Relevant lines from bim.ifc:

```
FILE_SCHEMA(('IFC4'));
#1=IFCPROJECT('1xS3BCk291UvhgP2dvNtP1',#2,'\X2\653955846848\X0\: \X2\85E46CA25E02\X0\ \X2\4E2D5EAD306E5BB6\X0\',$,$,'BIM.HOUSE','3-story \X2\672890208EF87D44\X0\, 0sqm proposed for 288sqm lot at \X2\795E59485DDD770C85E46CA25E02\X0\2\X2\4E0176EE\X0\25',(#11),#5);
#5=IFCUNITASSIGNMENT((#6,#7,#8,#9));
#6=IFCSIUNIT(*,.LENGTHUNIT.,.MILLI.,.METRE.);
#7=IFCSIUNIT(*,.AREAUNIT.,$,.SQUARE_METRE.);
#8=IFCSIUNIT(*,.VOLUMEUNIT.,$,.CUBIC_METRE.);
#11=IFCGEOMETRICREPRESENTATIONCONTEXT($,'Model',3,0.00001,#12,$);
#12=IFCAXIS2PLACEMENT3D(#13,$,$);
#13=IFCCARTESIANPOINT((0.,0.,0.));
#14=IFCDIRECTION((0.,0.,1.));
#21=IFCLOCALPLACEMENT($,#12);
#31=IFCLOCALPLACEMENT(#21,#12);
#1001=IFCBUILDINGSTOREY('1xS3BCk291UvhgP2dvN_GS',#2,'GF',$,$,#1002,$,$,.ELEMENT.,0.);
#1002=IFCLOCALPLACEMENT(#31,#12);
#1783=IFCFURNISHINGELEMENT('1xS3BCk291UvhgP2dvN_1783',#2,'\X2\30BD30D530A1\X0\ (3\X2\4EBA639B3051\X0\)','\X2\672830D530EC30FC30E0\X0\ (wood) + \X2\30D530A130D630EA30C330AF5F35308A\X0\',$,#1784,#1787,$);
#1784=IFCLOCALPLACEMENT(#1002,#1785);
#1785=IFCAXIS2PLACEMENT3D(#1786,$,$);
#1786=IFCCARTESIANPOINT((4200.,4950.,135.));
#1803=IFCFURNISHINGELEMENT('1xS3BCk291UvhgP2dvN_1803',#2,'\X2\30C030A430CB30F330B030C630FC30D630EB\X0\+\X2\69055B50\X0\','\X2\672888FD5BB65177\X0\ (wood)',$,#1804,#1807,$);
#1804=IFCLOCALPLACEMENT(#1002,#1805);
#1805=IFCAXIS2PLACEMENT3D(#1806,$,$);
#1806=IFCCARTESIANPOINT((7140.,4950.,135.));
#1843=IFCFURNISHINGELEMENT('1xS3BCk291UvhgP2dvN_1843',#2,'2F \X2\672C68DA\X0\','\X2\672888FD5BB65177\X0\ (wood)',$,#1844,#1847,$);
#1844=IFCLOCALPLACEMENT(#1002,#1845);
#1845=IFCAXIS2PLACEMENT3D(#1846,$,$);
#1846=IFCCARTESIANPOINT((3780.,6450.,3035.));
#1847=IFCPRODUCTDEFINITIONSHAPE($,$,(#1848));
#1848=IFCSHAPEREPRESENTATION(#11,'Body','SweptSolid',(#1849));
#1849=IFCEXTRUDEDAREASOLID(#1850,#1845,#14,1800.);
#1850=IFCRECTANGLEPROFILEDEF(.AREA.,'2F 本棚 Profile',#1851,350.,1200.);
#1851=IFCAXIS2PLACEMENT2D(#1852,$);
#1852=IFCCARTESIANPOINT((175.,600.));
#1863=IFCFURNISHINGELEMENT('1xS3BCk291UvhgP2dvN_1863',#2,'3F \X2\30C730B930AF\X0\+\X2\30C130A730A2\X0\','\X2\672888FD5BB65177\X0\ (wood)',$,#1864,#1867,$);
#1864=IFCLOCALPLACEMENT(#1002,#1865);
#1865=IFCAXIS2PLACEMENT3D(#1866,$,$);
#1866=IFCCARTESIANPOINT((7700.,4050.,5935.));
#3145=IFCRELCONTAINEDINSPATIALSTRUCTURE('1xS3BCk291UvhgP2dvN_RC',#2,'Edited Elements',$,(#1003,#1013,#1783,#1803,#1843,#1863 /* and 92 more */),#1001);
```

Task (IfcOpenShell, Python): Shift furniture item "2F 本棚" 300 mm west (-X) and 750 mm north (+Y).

```python
import ifcopenshell
import ifcopenshell.api.geometry
import ifcopenshell.util.placement
import ifcopenshell.util.unit

model = ifcopenshell.open("bim.ifc")
unit_scale = ifcopenshell.util.unit.calculate_unit_scale(model)

item = model.by_id(1843)
matrix = ifcopenshell.util.placement.get_local_placement(item.ObjectPlacement)
matrix[0, 3] -= 0.3 / unit_scale
matrix[1, 3] += 0.75 / unit_scale
ifcopenshell.api.geometry.edit_object_placement(model, product=item, matrix=matrix, is_si=False)

print(ifcopenshell.util.placement.get_local_placement(item.ObjectPlacement).round(3) + 0.0)

model.write("bim_updated.ifc")
```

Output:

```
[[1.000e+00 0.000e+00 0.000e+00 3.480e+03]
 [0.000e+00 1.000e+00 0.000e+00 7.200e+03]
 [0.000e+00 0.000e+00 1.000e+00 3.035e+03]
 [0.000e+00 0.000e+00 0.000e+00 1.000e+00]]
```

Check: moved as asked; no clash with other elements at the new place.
